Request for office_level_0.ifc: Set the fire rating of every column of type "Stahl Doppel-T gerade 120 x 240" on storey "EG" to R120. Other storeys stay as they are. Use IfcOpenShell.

First a look at what the model holds.

```python
import ifcopenshell
import ifcopenshell.util.element

model = ifcopenshell.open("office_level_0.ifc")
print(model.schema)
storey = next(s for s in model.by_type("IfcBuildingStorey") if s.Name == "EG")
columns = [e for e in ifcopenshell.util.element.get_decomposition(storey) if e.is_a("IfcColumn")]
seen = {}
for e in columns:
    element_type = ifcopenshell.util.element.get_type(e)
    key = (element_type.Name if element_type != e and element_type else None, ifcopenshell.util.element.get_pset(e, "Pset_ColumnCommon", "FireRating"))
    seen[key] = seen.get(key, 0) + 1
for (name, value), count in sorted(seen.items(), key=str):
    print(count, "x", name, "|", value)
```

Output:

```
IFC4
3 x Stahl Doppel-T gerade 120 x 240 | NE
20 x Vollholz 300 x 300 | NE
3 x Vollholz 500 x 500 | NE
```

```python
import ifcopenshell
import ifcopenshell.api.pset
import ifcopenshell.util.element

model = ifcopenshell.open("office_level_0.ifc")

storey = next(s for s in model.by_type("IfcBuildingStorey") if s.Name == "EG")
columns = [e for e in ifcopenshell.util.element.get_decomposition(storey) if e.is_a("IfcColumn")]

count = 0
for e in columns:
    element_type = ifcopenshell.util.element.get_type(e)
    if element_type in (None, e) or element_type.Name != "Stahl Doppel-T gerade 120 x 240":
        continue
    # add_pset returns the element's existing set when there is one.
    pset = ifcopenshell.api.pset.add_pset(model, product=e, name="Pset_ColumnCommon")
    ifcopenshell.api.pset.edit_pset(model, pset=pset, properties={"FireRating": "R120"})
    count += 1

print(count, "columns updated")

model.write("office_level_0_v2.ifc")
```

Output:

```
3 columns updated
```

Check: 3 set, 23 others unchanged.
